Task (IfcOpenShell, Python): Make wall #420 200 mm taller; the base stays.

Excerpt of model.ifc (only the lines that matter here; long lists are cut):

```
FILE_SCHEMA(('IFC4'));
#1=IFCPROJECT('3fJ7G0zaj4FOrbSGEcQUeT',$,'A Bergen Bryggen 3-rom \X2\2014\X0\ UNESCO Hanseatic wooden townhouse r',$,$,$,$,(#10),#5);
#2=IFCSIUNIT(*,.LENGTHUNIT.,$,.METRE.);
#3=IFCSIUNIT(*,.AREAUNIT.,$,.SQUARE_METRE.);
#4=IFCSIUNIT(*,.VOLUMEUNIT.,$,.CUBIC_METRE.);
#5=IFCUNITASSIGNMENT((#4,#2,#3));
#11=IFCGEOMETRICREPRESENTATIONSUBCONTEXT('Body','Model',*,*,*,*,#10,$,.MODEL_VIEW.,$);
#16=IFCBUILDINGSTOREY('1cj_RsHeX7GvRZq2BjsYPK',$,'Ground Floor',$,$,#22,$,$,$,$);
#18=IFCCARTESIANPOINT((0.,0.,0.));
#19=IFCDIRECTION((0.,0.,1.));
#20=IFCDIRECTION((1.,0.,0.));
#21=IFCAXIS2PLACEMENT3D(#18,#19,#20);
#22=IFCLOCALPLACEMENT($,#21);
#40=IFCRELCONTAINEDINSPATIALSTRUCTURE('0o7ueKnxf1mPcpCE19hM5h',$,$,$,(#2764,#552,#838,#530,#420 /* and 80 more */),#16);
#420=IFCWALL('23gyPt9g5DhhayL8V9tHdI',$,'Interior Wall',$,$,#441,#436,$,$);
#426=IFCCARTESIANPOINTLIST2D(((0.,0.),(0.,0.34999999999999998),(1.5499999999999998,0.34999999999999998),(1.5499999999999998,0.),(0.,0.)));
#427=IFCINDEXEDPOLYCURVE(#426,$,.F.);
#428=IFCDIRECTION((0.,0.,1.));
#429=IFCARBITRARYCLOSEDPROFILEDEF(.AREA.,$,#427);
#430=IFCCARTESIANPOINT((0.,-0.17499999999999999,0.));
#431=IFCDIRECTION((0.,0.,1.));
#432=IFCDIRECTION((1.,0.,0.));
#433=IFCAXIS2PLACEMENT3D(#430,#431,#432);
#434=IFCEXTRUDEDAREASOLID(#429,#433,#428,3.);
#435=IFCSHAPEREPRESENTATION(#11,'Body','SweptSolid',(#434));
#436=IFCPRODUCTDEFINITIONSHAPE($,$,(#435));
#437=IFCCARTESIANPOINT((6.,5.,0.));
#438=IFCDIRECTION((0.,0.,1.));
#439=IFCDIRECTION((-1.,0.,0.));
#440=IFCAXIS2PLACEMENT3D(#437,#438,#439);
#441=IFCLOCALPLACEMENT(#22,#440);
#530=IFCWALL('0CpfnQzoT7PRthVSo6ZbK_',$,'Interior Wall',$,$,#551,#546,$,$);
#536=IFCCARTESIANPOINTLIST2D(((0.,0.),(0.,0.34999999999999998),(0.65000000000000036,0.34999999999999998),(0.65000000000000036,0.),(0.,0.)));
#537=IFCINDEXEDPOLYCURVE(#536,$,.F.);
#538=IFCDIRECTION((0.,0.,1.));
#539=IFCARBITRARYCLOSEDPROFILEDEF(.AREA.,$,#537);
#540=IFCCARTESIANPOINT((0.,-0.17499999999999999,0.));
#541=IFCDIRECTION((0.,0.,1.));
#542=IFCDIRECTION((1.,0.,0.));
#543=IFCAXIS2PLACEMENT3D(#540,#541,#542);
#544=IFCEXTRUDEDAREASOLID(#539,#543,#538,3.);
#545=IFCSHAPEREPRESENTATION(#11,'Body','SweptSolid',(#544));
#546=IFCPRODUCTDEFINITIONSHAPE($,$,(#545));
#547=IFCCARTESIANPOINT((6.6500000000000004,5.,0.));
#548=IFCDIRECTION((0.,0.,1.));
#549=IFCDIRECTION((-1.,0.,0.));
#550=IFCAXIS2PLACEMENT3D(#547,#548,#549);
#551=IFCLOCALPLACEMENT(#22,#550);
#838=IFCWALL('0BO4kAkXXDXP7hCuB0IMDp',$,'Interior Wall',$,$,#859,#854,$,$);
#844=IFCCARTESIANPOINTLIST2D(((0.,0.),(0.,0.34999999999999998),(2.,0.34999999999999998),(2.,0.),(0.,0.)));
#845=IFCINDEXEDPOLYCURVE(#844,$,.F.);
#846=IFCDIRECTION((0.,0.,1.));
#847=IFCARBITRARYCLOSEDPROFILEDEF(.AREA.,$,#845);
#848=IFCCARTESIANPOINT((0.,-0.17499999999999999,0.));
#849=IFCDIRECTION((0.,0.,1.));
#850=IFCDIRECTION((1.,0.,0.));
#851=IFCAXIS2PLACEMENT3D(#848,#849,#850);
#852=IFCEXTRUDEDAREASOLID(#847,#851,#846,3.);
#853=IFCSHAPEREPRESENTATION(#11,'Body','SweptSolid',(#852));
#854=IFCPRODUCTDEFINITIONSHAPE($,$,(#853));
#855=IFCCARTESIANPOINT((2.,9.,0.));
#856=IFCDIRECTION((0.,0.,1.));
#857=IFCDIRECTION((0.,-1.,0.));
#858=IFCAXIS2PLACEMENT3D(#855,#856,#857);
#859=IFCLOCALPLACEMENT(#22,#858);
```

```python
import ifcopenshell
import ifcopenshell.geom
import ifcopenshell.util.representation
import ifcopenshell.util.shape
import ifcopenshell.util.unit

model = ifcopenshell.open("model.ifc")
unit_scale = ifcopenshell.util.unit.calculate_unit_scale(model)
settings = ifcopenshell.geom.settings()


def volume(element):
    """Net volume in cubic metres, openings subtracted."""
    shape = ifcopenshell.geom.create_shape(settings, element)
    return ifcopenshell.util.shape.get_volume(shape.geometry)


wall = model.by_guid("23gyPt9g5DhhayL8V9tHdI")
before = volume(wall)

body = ifcopenshell.util.representation.get_representation(wall, "Model", "Body")
solid = body.Items[0]
old_height = solid.Depth
solid.Depth += 0.2 / unit_scale
after = volume(wall)

print(f"height {old_height:g} -> {solid.Depth:g}, volume {before:.3f} -> {after:.3f} m3")

model.write("model_rev.ifc")
```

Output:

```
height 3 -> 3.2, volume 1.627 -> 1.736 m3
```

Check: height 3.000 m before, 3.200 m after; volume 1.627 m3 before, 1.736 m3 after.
